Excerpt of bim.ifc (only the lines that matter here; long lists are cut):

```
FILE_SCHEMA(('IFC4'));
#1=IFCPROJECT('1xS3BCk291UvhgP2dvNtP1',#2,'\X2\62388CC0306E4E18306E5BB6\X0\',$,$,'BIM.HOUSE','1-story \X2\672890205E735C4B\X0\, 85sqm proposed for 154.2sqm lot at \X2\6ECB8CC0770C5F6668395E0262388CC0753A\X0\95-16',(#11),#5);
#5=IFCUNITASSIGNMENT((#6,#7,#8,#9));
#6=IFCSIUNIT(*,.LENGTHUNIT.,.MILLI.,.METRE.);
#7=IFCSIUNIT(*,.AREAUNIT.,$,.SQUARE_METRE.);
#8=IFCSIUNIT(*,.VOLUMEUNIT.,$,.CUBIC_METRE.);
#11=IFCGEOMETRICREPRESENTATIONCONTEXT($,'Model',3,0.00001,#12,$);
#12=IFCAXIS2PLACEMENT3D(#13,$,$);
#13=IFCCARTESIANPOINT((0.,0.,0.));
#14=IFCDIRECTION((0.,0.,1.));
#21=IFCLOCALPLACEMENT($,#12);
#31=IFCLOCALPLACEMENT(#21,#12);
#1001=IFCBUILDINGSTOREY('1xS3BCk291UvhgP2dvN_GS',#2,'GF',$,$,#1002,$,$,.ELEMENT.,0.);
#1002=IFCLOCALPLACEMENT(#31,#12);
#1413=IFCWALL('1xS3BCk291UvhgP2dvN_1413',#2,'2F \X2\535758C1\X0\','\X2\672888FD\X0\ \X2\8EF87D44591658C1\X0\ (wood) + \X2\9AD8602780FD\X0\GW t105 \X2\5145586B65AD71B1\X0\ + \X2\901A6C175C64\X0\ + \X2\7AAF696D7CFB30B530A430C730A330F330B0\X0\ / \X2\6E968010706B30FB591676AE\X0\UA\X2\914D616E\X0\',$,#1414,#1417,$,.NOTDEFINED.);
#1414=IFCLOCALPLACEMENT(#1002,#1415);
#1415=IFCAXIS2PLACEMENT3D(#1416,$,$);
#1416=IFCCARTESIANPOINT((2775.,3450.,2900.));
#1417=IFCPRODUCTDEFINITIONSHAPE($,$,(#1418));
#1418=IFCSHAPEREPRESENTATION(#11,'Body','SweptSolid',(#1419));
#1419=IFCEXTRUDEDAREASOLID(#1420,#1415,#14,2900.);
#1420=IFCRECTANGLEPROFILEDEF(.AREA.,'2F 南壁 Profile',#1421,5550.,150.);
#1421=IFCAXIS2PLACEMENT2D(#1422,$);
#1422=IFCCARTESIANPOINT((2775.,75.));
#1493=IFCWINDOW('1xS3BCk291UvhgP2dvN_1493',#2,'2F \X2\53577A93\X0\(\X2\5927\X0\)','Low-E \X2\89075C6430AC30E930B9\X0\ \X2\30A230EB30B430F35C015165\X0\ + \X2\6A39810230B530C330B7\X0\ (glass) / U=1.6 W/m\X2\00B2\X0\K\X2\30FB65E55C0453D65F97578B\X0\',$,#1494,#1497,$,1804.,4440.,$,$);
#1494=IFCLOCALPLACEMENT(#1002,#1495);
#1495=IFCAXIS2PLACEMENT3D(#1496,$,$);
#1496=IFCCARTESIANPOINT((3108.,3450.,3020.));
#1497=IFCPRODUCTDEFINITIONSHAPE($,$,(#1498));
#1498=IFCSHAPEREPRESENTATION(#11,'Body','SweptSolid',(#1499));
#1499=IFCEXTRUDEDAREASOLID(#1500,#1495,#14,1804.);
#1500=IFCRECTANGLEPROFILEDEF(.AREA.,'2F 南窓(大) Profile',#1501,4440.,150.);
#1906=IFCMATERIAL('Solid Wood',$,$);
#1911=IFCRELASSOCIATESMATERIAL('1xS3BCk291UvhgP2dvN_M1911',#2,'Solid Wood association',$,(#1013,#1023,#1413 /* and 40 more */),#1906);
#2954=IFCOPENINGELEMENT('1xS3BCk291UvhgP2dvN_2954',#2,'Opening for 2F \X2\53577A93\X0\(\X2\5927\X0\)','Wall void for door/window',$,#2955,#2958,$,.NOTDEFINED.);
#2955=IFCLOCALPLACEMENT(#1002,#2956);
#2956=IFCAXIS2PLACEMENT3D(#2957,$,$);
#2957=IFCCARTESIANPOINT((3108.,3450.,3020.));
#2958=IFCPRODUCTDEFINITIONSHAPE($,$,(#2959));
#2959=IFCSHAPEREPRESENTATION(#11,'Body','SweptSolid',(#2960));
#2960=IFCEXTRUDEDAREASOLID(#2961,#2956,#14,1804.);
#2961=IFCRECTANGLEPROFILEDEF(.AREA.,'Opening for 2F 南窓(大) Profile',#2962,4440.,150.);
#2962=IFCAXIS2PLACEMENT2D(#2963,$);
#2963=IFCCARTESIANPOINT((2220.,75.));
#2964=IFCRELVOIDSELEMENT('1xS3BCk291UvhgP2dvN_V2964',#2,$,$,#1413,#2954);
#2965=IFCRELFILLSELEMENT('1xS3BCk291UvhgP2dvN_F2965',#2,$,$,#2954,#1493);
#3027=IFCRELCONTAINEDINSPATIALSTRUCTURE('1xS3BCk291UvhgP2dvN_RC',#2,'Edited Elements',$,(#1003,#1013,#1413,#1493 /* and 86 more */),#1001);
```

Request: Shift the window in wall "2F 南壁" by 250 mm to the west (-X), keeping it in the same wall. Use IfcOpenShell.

```python
import ifcopenshell
import ifcopenshell.api.geometry
import ifcopenshell.util.placement
import ifcopenshell.util.unit

model = ifcopenshell.open("bim.ifc")
unit_scale = ifcopenshell.util.unit.calculate_unit_scale(model)

window = model.by_id(1493)
opening = window.FillsVoids[0].RelatingOpeningElement
wall = opening.VoidsElements[0].RelatingBuildingElement

wall_matrix = ifcopenshell.util.placement.get_local_placement(wall.ObjectPlacement)
shift = wall_matrix[:3, 0] * -0.25 / unit_scale
before = ifcopenshell.util.placement.get_local_placement(window.ObjectPlacement)[:3, 3].copy()

# The window is not placed relative to its opening, so move both.
for product in (opening, window):
    matrix = ifcopenshell.util.placement.get_local_placement(product.ObjectPlacement)
    matrix[:3, 3] += shift
    ifcopenshell.api.geometry.edit_object_placement(model, product=product, matrix=matrix, is_si=False)

after = ifcopenshell.util.placement.get_local_placement(window.ObjectPlacement)[:3, 3]
print("window moved by", (after - before).round(3) + 0.0)

model.write("bim_updated.ifc")
```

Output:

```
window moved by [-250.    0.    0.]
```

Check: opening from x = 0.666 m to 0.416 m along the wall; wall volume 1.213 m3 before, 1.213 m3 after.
